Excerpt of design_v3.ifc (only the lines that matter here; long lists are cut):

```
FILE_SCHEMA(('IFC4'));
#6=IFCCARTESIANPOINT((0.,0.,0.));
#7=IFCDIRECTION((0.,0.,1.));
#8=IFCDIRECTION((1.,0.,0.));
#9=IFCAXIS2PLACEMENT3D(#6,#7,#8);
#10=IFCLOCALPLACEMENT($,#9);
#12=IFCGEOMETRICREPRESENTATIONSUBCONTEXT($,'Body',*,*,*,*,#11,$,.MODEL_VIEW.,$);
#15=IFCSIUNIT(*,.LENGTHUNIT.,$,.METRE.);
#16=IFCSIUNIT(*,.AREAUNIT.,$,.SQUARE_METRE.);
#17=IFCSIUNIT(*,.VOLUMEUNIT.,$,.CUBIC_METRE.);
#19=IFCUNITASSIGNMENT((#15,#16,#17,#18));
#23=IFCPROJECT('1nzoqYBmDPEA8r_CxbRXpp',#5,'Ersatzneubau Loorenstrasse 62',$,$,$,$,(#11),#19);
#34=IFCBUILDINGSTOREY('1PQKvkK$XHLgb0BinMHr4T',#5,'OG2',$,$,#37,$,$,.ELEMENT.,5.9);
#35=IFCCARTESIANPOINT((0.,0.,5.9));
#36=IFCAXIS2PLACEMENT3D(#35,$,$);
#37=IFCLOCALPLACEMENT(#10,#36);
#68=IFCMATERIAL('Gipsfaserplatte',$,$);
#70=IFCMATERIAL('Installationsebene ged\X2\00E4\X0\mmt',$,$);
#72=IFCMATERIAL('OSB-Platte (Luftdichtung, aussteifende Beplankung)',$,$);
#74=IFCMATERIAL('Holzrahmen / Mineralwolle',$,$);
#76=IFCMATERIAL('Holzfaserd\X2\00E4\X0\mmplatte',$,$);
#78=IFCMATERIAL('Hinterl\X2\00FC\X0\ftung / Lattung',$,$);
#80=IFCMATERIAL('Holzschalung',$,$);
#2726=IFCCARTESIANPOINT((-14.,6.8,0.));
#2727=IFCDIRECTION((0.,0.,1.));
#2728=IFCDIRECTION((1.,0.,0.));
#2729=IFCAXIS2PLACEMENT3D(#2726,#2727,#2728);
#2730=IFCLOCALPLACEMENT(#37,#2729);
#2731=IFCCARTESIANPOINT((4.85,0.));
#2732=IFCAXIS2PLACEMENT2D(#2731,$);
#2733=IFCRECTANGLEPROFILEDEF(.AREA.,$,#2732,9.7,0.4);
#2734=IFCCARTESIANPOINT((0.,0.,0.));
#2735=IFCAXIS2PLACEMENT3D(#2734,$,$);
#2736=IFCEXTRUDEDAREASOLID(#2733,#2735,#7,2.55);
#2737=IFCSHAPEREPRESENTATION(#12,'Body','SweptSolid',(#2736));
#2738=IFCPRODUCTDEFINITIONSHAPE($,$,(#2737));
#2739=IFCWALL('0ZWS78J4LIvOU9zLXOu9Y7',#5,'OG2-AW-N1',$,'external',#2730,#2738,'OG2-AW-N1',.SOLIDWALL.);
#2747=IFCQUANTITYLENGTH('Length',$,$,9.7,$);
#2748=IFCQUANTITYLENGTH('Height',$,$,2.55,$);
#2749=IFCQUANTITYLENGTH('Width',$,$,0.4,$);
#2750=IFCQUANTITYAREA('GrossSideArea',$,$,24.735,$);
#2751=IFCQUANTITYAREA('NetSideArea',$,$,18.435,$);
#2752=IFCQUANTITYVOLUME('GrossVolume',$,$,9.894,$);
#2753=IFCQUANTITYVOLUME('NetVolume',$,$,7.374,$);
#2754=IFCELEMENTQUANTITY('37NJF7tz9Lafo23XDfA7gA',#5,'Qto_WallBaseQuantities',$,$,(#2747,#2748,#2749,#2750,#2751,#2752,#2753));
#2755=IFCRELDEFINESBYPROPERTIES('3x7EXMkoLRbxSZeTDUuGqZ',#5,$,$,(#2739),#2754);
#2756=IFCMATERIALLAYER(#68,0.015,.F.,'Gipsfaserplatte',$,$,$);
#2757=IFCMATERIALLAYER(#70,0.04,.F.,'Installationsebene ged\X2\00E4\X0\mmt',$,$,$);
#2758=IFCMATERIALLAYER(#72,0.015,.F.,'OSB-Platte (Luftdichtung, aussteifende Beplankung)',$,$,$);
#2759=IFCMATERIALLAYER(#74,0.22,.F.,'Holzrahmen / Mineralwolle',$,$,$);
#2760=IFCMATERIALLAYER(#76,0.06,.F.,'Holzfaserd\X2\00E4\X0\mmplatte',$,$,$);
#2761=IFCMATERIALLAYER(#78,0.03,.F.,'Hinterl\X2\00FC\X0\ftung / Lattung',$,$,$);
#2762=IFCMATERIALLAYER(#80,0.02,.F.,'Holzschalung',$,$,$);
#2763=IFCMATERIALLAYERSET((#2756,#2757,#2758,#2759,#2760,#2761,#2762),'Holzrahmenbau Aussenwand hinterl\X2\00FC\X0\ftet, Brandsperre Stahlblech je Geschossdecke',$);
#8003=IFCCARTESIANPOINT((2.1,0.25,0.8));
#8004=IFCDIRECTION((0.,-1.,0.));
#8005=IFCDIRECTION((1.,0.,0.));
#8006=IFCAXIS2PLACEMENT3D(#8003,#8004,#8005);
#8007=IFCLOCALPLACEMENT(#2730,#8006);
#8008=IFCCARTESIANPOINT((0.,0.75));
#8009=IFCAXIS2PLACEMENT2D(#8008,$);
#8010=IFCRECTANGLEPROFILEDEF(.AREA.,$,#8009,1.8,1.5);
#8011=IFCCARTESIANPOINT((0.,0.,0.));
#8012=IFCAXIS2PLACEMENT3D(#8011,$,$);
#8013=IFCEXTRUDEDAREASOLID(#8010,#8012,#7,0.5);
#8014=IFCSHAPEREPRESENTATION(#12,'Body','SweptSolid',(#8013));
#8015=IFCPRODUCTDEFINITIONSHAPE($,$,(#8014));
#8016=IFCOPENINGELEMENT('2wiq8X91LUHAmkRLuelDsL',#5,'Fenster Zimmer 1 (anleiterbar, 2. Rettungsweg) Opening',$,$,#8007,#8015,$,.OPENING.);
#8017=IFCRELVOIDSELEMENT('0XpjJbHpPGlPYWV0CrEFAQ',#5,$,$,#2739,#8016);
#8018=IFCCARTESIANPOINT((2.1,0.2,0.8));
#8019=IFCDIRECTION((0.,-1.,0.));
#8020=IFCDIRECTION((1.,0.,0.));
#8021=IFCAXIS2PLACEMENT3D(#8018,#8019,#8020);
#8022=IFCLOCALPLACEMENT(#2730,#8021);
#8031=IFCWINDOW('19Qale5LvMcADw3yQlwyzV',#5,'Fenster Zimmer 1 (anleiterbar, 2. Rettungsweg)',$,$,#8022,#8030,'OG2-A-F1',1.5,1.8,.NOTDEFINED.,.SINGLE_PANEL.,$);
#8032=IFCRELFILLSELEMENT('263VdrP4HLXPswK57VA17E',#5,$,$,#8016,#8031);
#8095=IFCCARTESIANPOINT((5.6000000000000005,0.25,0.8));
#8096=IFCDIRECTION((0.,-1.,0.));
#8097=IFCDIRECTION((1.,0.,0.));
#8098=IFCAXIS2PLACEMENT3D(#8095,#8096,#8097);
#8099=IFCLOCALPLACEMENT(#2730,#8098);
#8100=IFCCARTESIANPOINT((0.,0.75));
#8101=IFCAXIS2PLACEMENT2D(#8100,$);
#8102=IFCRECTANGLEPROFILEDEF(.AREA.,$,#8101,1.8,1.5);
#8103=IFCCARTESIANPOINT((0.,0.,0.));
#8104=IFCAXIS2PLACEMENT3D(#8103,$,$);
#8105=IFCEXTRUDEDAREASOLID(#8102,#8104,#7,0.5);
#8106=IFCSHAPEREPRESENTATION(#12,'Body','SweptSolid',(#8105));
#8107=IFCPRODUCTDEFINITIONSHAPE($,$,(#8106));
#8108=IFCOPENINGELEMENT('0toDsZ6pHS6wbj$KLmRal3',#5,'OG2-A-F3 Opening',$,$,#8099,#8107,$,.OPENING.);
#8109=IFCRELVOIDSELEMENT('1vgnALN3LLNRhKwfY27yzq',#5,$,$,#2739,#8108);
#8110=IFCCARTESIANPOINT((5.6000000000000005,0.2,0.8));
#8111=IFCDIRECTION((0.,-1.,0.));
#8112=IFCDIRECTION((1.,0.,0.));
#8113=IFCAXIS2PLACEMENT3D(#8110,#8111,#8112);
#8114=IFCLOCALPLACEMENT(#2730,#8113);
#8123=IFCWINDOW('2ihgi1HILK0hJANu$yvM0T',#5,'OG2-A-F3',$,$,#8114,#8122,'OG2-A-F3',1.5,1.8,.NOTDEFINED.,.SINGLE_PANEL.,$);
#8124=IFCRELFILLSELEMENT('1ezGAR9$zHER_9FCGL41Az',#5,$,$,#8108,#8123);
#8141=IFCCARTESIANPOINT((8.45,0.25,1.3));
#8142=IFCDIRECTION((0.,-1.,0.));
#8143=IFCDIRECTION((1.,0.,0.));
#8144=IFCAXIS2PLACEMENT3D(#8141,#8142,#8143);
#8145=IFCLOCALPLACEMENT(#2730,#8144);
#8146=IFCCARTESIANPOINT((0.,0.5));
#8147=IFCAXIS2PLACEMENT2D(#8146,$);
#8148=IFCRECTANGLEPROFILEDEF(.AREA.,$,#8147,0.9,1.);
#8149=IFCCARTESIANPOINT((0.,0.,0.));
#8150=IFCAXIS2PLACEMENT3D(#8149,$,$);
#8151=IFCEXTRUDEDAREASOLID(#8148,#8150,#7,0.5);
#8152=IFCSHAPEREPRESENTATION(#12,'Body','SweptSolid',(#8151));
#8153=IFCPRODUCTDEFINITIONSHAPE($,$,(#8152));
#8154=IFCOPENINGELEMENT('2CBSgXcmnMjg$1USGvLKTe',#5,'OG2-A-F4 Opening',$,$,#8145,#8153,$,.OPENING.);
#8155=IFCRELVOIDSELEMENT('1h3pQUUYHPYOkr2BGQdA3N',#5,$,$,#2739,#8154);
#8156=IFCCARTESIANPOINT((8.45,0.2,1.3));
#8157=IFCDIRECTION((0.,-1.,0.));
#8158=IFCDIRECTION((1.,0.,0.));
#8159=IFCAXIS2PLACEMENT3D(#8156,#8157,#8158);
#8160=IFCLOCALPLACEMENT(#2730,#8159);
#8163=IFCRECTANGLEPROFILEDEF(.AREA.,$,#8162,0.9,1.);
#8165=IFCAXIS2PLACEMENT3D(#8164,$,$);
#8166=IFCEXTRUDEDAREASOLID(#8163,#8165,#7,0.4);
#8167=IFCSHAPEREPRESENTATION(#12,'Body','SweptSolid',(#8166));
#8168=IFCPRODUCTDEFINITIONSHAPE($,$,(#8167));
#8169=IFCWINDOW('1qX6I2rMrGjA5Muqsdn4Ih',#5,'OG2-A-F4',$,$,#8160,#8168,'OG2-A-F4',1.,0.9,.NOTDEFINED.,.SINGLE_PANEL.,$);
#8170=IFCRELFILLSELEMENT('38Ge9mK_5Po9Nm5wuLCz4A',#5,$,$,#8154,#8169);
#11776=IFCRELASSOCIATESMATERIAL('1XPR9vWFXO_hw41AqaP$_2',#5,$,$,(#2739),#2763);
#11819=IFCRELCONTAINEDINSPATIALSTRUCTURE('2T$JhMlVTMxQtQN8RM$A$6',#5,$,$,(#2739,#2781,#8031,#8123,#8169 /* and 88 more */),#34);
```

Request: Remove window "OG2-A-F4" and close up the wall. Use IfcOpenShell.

```python
import ifcopenshell
import ifcopenshell.api.feature
import ifcopenshell.api.pset
import ifcopenshell.api.root
import ifcopenshell.geom
import ifcopenshell.util.element
import ifcopenshell.util.shape
import ifcopenshell.util.unit

model = ifcopenshell.open("design_v3.ifc")
area_scale = ifcopenshell.util.unit.calculate_unit_scale(model, "AREAUNIT")
volume_scale = ifcopenshell.util.unit.calculate_unit_scale(model, "VOLUMEUNIT")
settings = ifcopenshell.geom.settings()


def volume(element):
    """Net volume in cubic metres, openings subtracted."""
    shape = ifcopenshell.geom.create_shape(settings, element)
    return ifcopenshell.util.shape.get_volume(shape.geometry)


window = model.by_guid("1qX6I2rMrGjA5Muqsdn4Ih")
opening = window.FillsVoids[0].RelatingOpeningElement
wall = opening.VoidsElements[0].RelatingBuildingElement
before = volume(wall)

ifcopenshell.api.root.remove_product(model, product=window)
ifcopenshell.api.feature.remove_feature(model, feature=opening)

after = volume(wall)
thickness = 0.4  # wall thickness in metres

# Update the wall's stored quantities.
qto = model.by_id(ifcopenshell.util.element.get_pset(wall, "Qto_WallBaseQuantities", should_inherit=False)["id"])
ifcopenshell.api.pset.edit_qto(model, qto=qto, properties={
    "NetSideArea": after / thickness / area_scale,
    "NetVolume": after / volume_scale,
})

print(f"wall volume {before:.3f} -> {after:.3f} m3")

model.write("design_v3_v2.ifc")
```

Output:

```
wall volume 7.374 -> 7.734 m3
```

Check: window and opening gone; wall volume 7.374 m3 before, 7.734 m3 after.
